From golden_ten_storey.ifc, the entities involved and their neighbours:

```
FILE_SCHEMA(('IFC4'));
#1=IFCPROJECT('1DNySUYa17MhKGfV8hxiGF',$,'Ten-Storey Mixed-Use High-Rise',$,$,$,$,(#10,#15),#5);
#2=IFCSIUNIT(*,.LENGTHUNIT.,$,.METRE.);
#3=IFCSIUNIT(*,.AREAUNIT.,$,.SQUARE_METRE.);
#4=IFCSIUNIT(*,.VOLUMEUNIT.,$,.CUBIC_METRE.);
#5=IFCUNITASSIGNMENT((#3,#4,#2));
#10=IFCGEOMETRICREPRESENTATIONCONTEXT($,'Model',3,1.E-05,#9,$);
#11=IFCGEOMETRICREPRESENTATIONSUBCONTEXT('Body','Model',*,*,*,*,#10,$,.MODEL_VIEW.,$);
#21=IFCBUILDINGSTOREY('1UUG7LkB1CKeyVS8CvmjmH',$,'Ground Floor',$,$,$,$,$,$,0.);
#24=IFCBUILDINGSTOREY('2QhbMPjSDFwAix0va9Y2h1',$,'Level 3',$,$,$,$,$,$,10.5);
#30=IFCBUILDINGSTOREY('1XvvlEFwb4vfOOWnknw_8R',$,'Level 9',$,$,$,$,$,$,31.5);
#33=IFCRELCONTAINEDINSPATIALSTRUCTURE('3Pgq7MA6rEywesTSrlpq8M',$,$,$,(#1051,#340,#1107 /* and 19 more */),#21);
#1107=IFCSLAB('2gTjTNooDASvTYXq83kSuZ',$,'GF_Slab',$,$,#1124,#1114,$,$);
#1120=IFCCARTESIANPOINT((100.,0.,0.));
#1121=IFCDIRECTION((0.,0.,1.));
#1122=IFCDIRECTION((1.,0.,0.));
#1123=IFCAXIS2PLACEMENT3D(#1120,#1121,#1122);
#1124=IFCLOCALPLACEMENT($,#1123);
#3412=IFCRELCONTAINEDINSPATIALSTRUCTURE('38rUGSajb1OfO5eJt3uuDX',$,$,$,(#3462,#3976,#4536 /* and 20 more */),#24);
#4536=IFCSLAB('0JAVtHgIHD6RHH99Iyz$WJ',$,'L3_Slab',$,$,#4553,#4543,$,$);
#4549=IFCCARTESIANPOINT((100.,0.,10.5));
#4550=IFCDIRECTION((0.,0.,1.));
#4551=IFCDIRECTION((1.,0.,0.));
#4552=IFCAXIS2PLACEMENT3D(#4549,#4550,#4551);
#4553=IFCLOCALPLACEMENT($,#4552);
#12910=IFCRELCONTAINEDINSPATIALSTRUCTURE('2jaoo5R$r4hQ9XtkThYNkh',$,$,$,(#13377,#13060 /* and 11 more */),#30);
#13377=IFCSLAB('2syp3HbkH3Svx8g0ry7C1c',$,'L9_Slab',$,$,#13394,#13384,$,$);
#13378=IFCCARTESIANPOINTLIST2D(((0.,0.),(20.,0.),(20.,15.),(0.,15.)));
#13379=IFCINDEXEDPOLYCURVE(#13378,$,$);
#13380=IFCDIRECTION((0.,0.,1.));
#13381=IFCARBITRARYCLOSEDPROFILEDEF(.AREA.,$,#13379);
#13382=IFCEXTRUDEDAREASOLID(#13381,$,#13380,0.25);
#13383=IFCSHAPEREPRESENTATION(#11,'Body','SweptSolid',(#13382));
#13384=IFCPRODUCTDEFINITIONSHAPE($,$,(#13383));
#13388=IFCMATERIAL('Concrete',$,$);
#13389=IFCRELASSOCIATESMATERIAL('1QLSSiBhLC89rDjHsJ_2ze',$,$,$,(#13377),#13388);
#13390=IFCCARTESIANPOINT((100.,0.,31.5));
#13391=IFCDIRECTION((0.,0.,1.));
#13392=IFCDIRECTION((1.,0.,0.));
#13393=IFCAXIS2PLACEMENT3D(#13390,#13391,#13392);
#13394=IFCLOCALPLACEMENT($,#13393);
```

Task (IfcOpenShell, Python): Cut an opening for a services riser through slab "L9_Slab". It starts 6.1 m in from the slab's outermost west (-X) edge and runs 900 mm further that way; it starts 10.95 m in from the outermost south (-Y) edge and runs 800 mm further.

```python
import numpy as np
import ifcopenshell
import ifcopenshell.api.feature
import ifcopenshell.api.geometry
import ifcopenshell.api.root
import ifcopenshell.geom
import ifcopenshell.util.placement
import ifcopenshell.util.representation
import ifcopenshell.util.shape
import ifcopenshell.util.unit

model = ifcopenshell.open("golden_ten_storey.ifc")
unit_scale = ifcopenshell.util.unit.calculate_unit_scale(model)
settings = ifcopenshell.geom.settings()


def volume(element):
    """Net volume in cubic metres, openings subtracted."""
    shape = ifcopenshell.geom.create_shape(settings, element)
    return ifcopenshell.util.shape.get_volume(shape.geometry)


slab = model.by_guid("2syp3HbkH3Svx8g0ry7C1c")
before = volume(slab)

# Extent in the slab's own axes, in metres. The edges named are its -X and -Y sides.
slab_shape = ifcopenshell.geom.create_shape(settings, slab)
vertices = ifcopenshell.util.shape.get_vertices(slab_shape.geometry)
x_min, y_min, bottom = vertices.min(axis=0)
top = vertices[:, 2].max()

opening = ifcopenshell.api.root.create_entity(model, ifc_class="IfcOpeningElement", name="Services riser opening", predefined_type="OPENING")
context = ifcopenshell.util.representation.get_context(model, "Model", "Body", "MODEL_VIEW")
width, depth = 0.9, 0.8
outline = [(0.0, 0.0), (width, 0.0), (width, depth), (0.0, depth), (0.0, 0.0)]
# Overshoot both faces by 50 mm so the cut is clean.
shape = ifcopenshell.api.geometry.add_slab_representation(
    model, context=context, depth=top - bottom + 0.1, polyline=outline
)
ifcopenshell.api.geometry.assign_representation(model, product=opening, representation=shape)

matrix = ifcopenshell.util.placement.get_local_placement(slab.ObjectPlacement)
matrix[:, 3] = matrix @ np.append(np.array([x_min + 6.1, y_min + 10.95, bottom - 0.05]) / unit_scale, 1.0)
ifcopenshell.api.geometry.edit_object_placement(model, product=opening, matrix=matrix, is_si=False)
ifcopenshell.api.feature.add_feature(model, feature=opening, element=slab)

after = volume(slab)

print(f"slab volume {before:.3f} -> {after:.3f} m3")

model.write("golden_ten_storey_updated.ifc")
```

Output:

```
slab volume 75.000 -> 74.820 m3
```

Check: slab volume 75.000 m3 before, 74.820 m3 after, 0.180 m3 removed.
